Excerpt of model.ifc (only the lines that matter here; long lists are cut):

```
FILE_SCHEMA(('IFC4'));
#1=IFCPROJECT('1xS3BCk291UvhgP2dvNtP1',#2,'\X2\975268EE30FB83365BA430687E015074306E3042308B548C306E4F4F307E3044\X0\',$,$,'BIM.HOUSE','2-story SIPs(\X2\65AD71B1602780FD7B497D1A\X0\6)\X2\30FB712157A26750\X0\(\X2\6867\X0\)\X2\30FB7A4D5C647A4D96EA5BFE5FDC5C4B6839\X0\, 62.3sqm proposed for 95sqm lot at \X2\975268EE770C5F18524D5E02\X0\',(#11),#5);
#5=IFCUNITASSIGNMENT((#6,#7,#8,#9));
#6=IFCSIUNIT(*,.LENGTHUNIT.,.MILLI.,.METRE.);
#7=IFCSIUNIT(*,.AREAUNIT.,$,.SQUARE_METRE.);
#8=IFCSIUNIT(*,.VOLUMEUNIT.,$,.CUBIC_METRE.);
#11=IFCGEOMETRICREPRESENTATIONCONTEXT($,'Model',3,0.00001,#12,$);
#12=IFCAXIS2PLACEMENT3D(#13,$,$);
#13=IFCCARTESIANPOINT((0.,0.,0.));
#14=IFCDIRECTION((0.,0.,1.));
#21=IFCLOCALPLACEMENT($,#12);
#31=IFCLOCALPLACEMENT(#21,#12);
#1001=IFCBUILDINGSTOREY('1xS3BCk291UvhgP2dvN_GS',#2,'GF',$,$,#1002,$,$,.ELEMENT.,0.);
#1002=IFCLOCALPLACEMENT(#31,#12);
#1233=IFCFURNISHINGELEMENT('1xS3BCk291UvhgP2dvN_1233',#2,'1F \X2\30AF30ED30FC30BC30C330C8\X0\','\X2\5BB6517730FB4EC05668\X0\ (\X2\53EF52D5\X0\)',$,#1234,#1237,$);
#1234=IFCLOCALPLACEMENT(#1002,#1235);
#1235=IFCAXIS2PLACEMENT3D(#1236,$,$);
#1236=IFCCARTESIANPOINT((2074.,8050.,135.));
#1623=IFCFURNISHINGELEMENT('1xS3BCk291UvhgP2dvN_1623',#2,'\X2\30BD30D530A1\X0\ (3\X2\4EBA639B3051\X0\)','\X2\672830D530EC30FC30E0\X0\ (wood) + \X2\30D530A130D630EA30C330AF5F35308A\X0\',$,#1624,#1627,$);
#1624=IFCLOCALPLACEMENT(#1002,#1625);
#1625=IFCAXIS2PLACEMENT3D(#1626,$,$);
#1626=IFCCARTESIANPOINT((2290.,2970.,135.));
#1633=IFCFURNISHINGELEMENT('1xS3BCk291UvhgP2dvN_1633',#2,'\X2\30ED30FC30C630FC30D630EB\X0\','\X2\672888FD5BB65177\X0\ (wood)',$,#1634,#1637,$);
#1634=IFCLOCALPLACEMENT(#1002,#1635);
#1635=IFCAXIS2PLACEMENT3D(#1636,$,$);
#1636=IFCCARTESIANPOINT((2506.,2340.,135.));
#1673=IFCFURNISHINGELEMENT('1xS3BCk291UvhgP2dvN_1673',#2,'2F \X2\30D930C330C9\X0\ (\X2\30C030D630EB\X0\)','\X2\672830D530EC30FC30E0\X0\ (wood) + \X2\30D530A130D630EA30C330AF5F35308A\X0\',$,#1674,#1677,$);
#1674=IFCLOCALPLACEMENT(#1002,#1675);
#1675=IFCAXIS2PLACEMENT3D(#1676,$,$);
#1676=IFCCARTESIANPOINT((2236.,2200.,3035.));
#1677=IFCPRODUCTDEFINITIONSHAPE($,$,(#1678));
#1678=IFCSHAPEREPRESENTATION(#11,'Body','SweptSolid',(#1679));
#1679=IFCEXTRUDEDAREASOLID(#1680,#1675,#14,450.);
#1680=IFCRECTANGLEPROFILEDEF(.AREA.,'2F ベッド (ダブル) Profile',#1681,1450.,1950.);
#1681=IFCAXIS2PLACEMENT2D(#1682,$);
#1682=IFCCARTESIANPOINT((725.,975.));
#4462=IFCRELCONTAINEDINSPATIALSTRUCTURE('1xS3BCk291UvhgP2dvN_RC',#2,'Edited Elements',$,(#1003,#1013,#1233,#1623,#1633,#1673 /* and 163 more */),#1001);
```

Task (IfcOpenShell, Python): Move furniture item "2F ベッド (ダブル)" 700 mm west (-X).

```python
import ifcopenshell
import ifcopenshell.api.geometry
import ifcopenshell.util.placement
import ifcopenshell.util.unit

model = ifcopenshell.open("model.ifc")
unit_scale = ifcopenshell.util.unit.calculate_unit_scale(model)

item = model.by_guid("1xS3BCk291UvhgP2dvN_1673")
matrix = ifcopenshell.util.placement.get_local_placement(item.ObjectPlacement)
matrix[0, 3] -= 0.7 / unit_scale
ifcopenshell.api.geometry.edit_object_placement(model, product=item, matrix=matrix, is_si=False)

print(ifcopenshell.util.placement.get_local_placement(item.ObjectPlacement).round(3) + 0.0)

model.write("model_rev.ifc")
```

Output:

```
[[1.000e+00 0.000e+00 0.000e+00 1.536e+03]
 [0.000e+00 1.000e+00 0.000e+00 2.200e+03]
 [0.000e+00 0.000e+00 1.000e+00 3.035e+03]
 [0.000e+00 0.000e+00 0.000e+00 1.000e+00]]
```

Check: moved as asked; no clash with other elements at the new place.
